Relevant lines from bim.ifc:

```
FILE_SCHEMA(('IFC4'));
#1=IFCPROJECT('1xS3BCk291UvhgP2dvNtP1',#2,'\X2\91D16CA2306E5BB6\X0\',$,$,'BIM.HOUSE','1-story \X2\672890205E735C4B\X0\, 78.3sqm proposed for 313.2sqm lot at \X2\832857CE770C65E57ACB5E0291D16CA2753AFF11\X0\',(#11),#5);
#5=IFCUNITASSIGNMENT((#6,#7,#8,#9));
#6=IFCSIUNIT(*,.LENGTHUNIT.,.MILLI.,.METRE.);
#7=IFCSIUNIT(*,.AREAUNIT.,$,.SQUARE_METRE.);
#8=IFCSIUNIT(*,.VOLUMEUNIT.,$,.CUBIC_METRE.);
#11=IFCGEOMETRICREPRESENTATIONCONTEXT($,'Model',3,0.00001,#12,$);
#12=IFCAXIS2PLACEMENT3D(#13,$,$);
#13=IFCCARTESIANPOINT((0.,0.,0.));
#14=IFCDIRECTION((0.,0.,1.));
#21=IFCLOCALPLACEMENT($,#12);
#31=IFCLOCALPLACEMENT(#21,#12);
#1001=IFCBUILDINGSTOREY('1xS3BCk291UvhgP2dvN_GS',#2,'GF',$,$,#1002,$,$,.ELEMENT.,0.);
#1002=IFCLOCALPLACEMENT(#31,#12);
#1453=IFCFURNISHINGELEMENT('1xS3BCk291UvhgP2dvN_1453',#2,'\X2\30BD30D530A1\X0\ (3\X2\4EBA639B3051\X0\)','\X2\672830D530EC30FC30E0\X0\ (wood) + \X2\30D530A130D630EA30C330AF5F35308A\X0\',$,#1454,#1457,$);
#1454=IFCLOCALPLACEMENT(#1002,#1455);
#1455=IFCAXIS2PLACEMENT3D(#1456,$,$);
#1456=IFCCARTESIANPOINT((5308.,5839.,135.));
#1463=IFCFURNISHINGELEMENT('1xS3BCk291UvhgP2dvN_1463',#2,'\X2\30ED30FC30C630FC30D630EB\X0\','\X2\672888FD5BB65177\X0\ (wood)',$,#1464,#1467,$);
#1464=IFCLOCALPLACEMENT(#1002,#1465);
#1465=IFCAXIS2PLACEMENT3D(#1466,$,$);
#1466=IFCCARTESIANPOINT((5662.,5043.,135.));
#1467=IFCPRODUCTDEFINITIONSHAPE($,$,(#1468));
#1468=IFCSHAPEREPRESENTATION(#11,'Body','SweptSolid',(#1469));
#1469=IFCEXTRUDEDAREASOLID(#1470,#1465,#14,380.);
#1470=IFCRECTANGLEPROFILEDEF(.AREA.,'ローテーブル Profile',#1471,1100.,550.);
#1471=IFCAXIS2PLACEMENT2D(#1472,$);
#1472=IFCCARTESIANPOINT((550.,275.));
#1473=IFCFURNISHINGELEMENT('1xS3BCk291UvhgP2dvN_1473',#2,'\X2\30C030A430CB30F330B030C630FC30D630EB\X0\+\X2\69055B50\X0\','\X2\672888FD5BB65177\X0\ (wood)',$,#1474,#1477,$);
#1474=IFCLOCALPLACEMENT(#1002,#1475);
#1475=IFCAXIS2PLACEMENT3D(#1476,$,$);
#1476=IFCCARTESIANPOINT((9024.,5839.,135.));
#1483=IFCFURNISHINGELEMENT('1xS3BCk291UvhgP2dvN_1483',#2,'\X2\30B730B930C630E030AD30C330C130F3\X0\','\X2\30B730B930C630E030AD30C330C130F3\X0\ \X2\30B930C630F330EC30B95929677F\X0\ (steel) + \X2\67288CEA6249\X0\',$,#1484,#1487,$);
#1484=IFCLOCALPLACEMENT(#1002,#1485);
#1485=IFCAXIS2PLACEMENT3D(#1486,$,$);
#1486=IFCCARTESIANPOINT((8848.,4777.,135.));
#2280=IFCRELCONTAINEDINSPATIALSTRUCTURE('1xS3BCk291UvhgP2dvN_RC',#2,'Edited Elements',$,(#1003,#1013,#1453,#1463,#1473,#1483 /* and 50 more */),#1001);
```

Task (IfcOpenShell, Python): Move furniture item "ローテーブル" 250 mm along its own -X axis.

```python
import ifcopenshell
import ifcopenshell.api.geometry
import ifcopenshell.util.placement

model = ifcopenshell.open("bim.ifc")

item = model.by_id(1463)
matrix = ifcopenshell.util.placement.get_local_placement(item.ObjectPlacement)
matrix[:3, 3] -= matrix[:3, 0] * 250.0
ifcopenshell.api.geometry.edit_object_placement(model, product=item, matrix=matrix, is_si=False)

print(ifcopenshell.util.placement.get_local_placement(item.ObjectPlacement).round(3) + 0.0)

model.write("bim_edited.ifc")
```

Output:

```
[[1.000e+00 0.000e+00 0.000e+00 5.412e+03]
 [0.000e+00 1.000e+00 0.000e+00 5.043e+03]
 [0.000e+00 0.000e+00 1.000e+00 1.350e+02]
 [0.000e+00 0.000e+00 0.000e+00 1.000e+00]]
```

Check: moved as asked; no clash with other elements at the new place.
